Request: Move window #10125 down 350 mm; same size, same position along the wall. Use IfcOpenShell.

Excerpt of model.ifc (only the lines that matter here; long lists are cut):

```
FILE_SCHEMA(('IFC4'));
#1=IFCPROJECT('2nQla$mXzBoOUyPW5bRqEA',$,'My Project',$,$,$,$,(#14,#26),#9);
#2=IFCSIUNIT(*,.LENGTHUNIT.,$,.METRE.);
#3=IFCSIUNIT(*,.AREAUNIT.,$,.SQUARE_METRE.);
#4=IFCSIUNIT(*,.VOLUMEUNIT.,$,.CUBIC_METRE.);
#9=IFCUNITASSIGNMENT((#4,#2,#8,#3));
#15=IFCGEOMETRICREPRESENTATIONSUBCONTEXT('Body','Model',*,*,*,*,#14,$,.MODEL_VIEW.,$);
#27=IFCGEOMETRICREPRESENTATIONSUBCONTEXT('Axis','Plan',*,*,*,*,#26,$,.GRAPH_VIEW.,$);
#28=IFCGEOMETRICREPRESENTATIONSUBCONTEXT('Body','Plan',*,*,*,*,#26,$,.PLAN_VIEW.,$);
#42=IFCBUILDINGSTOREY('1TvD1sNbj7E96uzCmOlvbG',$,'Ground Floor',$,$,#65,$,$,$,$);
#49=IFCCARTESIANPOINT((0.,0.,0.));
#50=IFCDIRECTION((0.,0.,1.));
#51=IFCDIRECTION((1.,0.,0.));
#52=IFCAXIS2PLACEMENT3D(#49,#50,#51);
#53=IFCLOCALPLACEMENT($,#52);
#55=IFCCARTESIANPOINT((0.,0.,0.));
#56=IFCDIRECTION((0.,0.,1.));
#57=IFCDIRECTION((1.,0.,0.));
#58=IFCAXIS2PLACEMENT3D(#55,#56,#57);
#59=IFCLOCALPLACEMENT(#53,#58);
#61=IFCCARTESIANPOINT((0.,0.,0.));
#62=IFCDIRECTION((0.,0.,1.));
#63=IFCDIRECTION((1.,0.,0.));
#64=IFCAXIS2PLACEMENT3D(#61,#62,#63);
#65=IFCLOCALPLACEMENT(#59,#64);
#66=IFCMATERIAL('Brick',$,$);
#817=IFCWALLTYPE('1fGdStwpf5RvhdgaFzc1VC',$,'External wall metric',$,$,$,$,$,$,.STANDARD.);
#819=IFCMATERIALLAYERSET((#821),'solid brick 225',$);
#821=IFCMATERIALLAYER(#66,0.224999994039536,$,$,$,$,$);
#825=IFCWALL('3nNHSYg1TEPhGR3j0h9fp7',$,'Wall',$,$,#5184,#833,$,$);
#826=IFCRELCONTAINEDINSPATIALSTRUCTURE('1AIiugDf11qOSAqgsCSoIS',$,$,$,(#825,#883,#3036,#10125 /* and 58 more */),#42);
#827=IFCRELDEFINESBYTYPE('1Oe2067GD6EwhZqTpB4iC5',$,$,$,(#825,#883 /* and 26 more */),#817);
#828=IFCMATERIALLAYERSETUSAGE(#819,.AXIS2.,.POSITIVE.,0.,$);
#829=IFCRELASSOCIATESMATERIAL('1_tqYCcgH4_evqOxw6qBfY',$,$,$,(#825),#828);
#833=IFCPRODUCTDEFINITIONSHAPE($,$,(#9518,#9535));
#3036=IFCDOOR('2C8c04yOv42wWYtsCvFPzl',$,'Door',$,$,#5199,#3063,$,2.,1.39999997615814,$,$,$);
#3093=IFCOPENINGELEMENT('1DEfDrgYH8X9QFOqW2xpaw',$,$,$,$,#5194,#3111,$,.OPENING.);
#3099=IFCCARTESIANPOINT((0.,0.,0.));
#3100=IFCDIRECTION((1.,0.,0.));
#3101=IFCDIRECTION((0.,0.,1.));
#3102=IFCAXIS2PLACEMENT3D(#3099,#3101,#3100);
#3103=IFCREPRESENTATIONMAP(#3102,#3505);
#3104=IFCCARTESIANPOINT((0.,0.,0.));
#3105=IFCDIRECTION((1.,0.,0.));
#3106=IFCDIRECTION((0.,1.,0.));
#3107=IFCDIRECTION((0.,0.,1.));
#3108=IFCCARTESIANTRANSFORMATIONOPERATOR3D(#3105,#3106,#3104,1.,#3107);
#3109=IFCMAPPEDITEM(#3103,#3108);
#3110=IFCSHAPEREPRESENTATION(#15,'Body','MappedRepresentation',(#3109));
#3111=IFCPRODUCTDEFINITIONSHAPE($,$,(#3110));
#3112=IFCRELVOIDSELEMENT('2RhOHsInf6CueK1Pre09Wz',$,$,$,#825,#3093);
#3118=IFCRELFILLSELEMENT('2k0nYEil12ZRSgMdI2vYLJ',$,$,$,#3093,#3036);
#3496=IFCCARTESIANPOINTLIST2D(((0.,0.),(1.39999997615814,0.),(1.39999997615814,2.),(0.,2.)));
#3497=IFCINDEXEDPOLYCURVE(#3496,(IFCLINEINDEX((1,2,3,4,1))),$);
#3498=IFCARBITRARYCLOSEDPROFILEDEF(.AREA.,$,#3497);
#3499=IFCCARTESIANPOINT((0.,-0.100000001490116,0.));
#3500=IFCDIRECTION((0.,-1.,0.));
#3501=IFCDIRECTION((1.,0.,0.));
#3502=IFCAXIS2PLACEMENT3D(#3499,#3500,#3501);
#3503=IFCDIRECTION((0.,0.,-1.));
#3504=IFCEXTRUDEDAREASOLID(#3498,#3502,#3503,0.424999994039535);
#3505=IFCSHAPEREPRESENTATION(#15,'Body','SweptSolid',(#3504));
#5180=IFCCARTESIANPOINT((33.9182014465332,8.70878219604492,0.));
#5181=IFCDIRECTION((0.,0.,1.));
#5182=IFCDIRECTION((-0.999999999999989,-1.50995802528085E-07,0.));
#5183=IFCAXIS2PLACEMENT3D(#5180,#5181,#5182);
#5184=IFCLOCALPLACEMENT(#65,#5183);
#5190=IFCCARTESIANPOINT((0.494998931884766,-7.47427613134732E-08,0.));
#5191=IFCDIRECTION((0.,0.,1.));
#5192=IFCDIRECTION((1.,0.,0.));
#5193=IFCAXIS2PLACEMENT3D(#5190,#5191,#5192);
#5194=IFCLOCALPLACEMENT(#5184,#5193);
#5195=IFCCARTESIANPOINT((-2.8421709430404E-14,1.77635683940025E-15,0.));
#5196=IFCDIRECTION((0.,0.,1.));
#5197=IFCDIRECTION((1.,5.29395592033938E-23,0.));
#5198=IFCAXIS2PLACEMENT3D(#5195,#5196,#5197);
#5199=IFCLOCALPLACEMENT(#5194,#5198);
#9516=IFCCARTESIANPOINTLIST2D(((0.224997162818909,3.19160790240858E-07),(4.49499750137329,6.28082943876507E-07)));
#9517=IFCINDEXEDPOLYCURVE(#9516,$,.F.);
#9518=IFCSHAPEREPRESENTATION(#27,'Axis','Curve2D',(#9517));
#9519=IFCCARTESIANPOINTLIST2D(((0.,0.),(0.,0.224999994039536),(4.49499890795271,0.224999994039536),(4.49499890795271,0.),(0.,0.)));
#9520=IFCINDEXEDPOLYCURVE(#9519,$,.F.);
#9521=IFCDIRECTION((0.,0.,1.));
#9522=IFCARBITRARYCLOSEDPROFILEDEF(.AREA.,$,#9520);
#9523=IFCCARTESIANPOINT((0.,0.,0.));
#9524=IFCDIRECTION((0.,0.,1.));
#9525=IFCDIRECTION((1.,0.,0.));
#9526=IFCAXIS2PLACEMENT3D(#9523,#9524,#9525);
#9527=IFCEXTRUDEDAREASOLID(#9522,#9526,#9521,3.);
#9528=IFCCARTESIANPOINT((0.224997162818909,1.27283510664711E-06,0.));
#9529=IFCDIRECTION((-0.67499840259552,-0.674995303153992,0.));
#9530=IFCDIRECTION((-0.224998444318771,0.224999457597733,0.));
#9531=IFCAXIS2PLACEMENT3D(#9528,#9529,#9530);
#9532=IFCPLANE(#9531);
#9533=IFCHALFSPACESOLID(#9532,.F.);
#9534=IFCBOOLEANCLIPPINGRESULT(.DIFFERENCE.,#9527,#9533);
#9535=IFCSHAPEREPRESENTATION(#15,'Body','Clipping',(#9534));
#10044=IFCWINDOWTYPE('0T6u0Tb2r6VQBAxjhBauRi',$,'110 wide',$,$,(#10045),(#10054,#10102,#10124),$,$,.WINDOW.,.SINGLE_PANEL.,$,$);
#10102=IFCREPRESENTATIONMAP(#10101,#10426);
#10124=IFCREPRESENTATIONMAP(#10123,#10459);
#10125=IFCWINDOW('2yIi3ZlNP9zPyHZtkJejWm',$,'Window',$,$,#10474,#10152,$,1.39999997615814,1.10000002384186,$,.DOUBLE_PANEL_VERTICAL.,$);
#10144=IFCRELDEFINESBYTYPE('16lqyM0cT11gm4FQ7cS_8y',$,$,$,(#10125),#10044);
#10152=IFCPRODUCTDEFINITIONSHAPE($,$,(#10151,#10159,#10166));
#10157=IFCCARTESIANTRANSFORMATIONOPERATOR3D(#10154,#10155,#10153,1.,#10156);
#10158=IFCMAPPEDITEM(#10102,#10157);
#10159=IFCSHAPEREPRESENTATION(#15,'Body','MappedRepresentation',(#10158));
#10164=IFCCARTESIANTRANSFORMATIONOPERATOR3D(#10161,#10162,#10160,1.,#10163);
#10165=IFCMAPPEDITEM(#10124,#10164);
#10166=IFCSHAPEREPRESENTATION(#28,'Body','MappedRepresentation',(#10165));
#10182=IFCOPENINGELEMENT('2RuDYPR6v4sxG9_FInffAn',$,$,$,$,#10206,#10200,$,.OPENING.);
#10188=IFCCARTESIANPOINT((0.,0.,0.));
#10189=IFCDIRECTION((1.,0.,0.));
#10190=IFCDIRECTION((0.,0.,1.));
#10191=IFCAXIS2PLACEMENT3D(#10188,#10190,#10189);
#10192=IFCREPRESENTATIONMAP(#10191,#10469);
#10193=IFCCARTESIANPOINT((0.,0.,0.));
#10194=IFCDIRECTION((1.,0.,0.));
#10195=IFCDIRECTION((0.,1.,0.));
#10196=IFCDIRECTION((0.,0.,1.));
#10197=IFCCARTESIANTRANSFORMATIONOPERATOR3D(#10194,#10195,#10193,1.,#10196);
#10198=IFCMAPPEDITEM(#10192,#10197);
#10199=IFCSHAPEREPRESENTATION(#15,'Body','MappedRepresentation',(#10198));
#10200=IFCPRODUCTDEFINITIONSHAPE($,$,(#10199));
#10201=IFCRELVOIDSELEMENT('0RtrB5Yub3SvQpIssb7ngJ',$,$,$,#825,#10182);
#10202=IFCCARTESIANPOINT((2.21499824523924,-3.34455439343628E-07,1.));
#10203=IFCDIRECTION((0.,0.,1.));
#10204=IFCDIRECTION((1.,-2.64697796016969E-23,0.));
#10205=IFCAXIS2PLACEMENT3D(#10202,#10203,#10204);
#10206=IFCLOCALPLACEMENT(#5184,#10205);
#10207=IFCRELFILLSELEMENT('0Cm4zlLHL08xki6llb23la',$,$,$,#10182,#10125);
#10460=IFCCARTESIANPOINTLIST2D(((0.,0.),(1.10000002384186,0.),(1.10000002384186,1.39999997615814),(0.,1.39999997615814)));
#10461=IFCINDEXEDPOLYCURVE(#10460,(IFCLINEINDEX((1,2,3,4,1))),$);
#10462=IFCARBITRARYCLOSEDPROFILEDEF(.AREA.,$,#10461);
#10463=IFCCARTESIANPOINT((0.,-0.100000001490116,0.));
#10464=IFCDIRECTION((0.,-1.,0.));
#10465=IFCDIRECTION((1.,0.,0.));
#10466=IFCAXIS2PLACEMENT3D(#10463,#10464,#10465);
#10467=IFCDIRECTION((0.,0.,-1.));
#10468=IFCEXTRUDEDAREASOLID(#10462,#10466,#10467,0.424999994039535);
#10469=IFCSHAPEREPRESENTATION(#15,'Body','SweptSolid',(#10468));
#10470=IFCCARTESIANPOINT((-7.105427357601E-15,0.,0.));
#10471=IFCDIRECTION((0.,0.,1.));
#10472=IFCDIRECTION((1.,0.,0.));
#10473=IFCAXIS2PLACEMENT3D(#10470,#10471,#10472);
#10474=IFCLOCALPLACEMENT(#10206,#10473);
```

```python
import numpy as np
import ifcopenshell
import ifcopenshell.api.geometry
import ifcopenshell.util.placement
import ifcopenshell.util.unit

model = ifcopenshell.open("model.ifc")
unit_scale = ifcopenshell.util.unit.calculate_unit_scale(model)

window = model.by_guid("2yIi3ZlNP9zPyHZtkJejWm")
opening = window.FillsVoids[0].RelatingOpeningElement
dz = -0.35 / unit_scale

shift = np.array([0.0, 0.0, dz])
# The window is placed relative to its opening, so it follows when the opening moves.
matrix = ifcopenshell.util.placement.get_local_placement(opening.ObjectPlacement)
matrix[:3, 3] += shift
ifcopenshell.api.geometry.edit_object_placement(
    model, product=opening, matrix=matrix, is_si=False, should_transform_children=True
)

print(f"moved by {dz * unit_scale:+.3f} m")

model.write("model_v2.ifc")
```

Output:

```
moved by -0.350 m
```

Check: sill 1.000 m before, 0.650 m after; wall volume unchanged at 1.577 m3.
